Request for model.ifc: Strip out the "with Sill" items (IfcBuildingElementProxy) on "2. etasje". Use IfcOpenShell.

First a look at what the model holds.

```python
import ifcopenshell
import ifcopenshell.util.element

model = ifcopenshell.open("model.ifc")
print(model.schema)
storey = next(s for s in model.by_type("IfcBuildingStorey") if s.Name == "2. etasje")
proxies = [e for e in ifcopenshell.util.element.get_decomposition(storey) if e.is_a("IfcBuildingElementProxy")]
seen = {}
for e in proxies:
    element_type = ifcopenshell.util.element.get_type(e)
    name = element_type.Name if element_type not in (None, e) else None
    seen[name] = seen.get(name, 0) + 1
for name, count in sorted(seen.items(), key=str):
    print(count, "x", name)
```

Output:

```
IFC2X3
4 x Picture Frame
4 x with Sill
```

```python
import ifcopenshell
import ifcopenshell.api.root
import ifcopenshell.util.element

model = ifcopenshell.open("model.ifc")

storey = next(s for s in model.by_type("IfcBuildingStorey") if s.Name == "2. etasje")
proxies = [e for e in ifcopenshell.util.element.get_decomposition(storey) if e.is_a("IfcBuildingElementProxy")]
targets = [e for e in proxies if (t := ifcopenshell.util.element.get_type(e)) not in (None, e) and t.Name == "with Sill"]

for e in targets:
    ifcopenshell.api.root.remove_product(model, product=e)
print(len(targets), "removed")

model.write("model_edited.ifc")
```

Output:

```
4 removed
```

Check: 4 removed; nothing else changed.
